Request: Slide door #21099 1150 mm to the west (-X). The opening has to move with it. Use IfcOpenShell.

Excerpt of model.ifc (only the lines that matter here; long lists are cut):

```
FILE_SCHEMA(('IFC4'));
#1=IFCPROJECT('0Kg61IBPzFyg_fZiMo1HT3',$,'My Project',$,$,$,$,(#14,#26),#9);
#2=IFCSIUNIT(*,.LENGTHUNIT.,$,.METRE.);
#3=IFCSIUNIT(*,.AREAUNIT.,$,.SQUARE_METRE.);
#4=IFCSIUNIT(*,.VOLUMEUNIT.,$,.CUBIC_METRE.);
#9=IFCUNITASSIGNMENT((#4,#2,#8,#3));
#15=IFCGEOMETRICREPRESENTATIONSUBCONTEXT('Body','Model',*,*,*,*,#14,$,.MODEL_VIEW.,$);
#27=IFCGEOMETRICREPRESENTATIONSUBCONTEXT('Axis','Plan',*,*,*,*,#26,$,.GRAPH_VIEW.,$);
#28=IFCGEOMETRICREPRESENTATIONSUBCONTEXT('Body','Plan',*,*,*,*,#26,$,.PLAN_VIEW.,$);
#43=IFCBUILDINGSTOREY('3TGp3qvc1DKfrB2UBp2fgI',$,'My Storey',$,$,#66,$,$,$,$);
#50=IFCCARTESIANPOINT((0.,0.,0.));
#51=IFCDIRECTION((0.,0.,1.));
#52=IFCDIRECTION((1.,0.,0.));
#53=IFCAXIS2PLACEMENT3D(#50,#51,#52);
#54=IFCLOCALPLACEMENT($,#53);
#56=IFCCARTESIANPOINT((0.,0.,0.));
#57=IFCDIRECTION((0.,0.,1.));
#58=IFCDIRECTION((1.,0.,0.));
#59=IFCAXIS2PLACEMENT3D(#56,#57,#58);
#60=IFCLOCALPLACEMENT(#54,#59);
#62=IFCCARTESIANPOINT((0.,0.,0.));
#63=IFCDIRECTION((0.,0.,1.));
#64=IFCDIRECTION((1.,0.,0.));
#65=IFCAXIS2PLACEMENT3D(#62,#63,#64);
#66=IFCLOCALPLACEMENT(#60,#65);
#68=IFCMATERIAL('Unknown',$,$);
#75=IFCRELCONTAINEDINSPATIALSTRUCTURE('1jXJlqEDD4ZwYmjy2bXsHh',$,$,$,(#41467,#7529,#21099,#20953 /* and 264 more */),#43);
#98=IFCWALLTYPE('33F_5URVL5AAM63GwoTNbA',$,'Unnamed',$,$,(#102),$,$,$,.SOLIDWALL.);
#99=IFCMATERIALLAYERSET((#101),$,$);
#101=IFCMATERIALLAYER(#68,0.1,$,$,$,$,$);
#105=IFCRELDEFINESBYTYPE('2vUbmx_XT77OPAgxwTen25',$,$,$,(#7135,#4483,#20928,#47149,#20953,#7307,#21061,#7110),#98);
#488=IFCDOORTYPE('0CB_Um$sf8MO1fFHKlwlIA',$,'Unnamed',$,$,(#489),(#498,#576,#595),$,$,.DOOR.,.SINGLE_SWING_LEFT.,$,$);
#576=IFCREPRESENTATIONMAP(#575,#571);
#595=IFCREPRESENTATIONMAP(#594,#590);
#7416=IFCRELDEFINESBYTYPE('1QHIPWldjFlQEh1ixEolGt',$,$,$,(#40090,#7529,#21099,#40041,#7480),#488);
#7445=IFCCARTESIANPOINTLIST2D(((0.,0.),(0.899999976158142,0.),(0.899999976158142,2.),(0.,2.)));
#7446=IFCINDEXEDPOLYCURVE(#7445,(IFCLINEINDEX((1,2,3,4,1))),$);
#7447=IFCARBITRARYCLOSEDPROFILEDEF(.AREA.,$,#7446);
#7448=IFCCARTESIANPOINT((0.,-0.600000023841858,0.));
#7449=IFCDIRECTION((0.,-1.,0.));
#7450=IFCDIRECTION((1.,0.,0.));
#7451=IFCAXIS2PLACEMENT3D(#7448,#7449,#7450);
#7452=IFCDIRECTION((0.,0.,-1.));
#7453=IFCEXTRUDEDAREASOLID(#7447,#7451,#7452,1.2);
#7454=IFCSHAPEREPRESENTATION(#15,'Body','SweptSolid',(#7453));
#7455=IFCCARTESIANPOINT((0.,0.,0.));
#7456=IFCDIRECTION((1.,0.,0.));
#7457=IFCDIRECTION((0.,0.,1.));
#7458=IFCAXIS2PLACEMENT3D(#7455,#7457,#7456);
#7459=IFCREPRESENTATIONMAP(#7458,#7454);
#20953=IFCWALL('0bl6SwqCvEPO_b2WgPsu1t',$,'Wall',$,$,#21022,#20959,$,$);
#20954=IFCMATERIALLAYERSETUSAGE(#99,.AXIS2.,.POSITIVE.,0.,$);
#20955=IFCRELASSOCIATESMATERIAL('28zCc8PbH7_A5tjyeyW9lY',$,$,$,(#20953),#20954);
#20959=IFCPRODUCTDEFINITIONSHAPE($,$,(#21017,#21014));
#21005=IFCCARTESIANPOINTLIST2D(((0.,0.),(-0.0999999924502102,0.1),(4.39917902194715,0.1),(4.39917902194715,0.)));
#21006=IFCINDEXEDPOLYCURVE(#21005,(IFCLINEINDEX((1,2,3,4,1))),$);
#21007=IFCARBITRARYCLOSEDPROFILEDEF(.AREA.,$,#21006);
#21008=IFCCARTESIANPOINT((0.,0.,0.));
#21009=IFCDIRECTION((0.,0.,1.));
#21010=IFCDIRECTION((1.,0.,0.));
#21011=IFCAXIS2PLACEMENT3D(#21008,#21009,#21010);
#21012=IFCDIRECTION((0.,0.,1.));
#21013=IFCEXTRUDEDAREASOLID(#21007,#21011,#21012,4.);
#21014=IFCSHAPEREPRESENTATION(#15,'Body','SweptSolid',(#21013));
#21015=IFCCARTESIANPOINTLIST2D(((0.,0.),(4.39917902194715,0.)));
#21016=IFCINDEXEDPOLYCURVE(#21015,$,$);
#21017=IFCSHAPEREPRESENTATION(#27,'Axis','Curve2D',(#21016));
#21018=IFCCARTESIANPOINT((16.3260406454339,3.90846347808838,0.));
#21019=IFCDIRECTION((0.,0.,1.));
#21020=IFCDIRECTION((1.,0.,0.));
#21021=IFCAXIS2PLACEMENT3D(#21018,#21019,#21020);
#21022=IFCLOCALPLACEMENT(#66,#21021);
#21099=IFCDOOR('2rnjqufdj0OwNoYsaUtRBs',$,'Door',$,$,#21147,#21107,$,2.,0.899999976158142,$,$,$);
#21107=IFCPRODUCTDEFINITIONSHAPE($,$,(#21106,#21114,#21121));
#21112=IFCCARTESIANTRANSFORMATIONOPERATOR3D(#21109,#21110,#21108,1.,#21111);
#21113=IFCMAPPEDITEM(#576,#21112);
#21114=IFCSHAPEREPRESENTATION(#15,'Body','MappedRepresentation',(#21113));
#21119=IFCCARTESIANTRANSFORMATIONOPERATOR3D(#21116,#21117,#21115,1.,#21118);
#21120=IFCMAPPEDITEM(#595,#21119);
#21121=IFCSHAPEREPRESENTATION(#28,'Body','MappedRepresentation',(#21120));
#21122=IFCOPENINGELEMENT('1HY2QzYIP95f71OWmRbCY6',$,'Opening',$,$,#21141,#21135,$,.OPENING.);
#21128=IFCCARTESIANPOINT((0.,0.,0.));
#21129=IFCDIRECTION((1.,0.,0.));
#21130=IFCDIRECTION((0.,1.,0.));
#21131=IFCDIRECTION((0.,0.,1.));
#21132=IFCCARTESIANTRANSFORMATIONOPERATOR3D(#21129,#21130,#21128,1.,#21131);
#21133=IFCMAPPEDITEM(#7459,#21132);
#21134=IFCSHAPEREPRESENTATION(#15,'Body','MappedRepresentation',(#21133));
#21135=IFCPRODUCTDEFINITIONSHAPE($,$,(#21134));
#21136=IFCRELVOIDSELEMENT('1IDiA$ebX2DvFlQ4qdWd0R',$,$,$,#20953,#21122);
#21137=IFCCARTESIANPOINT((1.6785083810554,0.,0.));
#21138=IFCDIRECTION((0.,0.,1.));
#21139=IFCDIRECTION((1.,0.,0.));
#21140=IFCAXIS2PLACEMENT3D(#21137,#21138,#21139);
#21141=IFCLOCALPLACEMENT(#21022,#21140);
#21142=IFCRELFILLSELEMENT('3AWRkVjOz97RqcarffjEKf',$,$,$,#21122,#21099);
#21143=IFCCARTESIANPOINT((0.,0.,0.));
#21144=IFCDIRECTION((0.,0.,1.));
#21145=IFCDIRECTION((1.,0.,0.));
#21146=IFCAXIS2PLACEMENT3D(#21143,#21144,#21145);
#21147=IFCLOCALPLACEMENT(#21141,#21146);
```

```python
import ifcopenshell
import ifcopenshell.api.geometry
import ifcopenshell.util.placement
import ifcopenshell.util.unit

model = ifcopenshell.open("model.ifc")
unit_scale = ifcopenshell.util.unit.calculate_unit_scale(model)

door = model.by_guid("2rnjqufdj0OwNoYsaUtRBs")
opening = door.FillsVoids[0].RelatingOpeningElement
wall = opening.VoidsElements[0].RelatingBuildingElement

wall_matrix = ifcopenshell.util.placement.get_local_placement(wall.ObjectPlacement)
shift = wall_matrix[:3, 0] * -1.15 / unit_scale
before = ifcopenshell.util.placement.get_local_placement(door.ObjectPlacement)[:3, 3].copy()

# The door is placed relative to its opening, so it follows when the opening moves.
matrix = ifcopenshell.util.placement.get_local_placement(opening.ObjectPlacement)
matrix[:3, 3] += shift
ifcopenshell.api.geometry.edit_object_placement(
    model, product=opening, matrix=matrix, is_si=False, should_transform_children=True
)

after = ifcopenshell.util.placement.get_local_placement(door.ObjectPlacement)[:3, 3]
print("door moved by", (after - before).round(3) + 0.0)

model.write("model_updated.ifc")
```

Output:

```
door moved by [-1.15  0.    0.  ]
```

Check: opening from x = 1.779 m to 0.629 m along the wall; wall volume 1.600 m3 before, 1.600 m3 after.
